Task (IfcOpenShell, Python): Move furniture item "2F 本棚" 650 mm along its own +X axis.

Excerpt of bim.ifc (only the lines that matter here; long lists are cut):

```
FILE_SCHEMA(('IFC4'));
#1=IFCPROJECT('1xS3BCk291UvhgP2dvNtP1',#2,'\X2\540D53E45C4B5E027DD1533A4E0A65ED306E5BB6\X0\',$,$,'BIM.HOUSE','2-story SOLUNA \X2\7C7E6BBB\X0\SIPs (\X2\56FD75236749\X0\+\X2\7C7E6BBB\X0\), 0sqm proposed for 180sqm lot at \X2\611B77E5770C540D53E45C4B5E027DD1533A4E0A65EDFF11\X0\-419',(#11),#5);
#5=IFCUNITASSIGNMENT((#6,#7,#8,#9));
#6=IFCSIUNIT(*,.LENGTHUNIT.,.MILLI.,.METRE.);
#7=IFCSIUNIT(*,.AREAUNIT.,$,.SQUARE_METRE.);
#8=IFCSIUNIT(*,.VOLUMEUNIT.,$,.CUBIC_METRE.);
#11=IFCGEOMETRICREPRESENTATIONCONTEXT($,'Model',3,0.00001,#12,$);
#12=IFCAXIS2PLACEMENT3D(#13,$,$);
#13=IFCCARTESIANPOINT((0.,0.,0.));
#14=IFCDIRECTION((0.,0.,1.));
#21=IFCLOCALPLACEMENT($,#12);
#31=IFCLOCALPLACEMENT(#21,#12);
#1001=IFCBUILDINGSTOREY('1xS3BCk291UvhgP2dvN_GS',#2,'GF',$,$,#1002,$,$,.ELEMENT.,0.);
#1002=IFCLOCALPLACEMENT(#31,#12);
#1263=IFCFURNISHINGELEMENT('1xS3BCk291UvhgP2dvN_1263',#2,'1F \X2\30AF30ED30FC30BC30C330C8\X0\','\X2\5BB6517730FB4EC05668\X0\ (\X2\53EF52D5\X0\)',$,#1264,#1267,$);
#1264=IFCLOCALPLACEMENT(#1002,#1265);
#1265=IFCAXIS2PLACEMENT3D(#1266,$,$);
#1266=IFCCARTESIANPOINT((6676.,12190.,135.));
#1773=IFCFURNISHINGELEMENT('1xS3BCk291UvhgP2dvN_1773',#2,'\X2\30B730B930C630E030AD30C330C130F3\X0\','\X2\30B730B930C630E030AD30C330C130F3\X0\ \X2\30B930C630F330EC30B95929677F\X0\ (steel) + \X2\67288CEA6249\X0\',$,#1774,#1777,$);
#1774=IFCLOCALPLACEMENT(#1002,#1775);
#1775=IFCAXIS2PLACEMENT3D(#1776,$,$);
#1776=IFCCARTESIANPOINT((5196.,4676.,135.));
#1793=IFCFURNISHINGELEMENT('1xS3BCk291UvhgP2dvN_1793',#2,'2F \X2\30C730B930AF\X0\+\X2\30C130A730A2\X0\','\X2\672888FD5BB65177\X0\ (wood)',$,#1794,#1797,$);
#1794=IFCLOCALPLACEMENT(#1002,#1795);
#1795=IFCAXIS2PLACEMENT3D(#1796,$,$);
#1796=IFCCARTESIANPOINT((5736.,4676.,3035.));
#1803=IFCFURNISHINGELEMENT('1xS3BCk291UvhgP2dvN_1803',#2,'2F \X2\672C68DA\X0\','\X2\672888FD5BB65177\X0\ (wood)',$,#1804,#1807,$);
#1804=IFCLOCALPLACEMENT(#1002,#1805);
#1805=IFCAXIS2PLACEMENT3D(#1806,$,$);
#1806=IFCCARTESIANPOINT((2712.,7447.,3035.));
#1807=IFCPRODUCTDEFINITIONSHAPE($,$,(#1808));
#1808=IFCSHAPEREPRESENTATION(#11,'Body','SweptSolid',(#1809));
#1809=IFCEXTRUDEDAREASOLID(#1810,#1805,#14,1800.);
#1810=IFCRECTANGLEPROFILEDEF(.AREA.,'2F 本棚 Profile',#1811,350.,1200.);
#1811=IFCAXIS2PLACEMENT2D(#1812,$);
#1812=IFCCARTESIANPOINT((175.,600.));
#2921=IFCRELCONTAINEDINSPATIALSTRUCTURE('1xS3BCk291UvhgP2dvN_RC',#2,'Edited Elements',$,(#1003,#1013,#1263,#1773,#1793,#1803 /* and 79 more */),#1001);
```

```python
import ifcopenshell
import ifcopenshell.api.geometry
import ifcopenshell.util.placement
import ifcopenshell.util.unit

model = ifcopenshell.open("bim.ifc")
unit_scale = ifcopenshell.util.unit.calculate_unit_scale(model)

item = model.by_guid("1xS3BCk291UvhgP2dvN_1803")
matrix = ifcopenshell.util.placement.get_local_placement(item.ObjectPlacement)
matrix[:3, 3] += matrix[:3, 0] * 0.65 / unit_scale
ifcopenshell.api.geometry.edit_object_placement(model, product=item, matrix=matrix, is_si=False)

print(ifcopenshell.util.placement.get_local_placement(item.ObjectPlacement).round(3) + 0.0)

model.write("bim_edited.ifc")
```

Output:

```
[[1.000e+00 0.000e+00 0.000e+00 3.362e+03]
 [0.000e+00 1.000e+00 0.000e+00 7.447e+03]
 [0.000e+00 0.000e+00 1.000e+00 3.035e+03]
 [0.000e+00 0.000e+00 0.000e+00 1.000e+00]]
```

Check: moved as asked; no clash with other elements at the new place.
